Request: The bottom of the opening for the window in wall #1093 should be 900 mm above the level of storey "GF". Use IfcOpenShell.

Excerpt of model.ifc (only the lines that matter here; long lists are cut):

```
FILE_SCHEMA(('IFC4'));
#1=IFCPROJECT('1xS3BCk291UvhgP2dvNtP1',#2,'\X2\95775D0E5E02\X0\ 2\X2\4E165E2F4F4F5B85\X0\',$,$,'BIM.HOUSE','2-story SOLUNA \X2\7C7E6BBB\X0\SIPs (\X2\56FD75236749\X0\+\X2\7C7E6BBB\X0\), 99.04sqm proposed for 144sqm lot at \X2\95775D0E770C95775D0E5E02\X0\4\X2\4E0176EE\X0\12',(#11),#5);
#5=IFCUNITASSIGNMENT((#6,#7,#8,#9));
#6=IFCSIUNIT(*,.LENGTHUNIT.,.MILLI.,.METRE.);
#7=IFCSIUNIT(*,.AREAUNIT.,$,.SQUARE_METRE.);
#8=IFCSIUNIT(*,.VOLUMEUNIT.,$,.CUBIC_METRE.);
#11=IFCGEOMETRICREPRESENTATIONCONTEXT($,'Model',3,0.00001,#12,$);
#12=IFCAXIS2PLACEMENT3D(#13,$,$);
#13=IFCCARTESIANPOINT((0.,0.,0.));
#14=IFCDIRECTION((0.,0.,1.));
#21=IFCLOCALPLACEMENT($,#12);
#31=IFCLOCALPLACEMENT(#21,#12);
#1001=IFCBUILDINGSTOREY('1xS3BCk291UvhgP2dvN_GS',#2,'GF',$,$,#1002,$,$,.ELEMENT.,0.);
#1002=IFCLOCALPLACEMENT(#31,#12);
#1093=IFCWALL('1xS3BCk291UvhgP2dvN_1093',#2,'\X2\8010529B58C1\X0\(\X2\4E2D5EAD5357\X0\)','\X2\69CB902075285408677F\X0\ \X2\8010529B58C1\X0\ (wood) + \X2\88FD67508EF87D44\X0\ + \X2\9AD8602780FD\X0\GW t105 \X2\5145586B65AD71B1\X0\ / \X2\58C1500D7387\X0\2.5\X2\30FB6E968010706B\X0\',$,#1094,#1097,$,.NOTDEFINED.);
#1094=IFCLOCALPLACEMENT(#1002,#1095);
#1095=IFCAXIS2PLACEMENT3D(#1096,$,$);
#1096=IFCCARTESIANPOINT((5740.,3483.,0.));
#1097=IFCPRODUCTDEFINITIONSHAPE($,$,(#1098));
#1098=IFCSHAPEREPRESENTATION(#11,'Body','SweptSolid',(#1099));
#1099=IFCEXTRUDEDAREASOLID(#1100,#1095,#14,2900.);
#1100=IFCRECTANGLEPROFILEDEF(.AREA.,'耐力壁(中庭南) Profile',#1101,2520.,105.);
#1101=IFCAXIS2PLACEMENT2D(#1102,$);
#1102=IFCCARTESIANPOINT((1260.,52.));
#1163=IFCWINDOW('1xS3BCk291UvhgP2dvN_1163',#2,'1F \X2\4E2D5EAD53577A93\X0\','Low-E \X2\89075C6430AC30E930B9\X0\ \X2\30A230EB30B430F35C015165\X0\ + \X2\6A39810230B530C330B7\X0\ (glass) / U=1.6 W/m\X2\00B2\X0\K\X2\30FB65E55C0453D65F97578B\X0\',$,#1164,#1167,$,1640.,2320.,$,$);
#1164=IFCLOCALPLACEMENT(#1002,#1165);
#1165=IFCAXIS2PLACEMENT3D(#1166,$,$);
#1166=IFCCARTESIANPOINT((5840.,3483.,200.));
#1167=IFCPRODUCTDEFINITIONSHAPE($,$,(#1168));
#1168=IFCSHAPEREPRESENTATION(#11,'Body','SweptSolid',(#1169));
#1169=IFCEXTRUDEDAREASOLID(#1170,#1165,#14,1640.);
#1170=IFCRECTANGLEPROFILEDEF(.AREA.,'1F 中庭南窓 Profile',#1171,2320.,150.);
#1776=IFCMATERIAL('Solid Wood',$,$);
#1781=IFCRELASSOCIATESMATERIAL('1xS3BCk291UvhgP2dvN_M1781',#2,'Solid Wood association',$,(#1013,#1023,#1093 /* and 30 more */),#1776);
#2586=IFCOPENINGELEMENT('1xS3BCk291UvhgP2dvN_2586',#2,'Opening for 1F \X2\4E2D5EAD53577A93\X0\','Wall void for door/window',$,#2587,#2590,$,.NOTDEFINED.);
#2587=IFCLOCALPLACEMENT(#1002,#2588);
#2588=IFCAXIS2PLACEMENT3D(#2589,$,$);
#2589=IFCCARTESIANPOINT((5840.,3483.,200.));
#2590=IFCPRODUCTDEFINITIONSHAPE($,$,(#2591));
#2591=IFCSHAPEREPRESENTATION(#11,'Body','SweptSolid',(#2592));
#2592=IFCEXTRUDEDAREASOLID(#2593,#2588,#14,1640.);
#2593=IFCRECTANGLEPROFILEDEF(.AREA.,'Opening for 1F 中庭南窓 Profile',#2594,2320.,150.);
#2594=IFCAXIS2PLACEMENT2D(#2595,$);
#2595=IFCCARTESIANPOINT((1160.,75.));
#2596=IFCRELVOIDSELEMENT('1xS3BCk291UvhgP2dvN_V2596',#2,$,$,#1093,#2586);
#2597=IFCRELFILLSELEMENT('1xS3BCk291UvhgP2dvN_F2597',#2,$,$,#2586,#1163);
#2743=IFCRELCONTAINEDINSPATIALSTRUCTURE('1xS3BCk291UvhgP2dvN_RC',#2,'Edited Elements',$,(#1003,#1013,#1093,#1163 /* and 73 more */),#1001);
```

```python
import numpy as np
import ifcopenshell
import ifcopenshell.api.geometry
import ifcopenshell.geom
import ifcopenshell.util.element
import ifcopenshell.util.placement
import ifcopenshell.util.shape
import ifcopenshell.util.unit

model = ifcopenshell.open("model.ifc")
unit_scale = ifcopenshell.util.unit.calculate_unit_scale(model)

window = model.by_guid("1xS3BCk291UvhgP2dvN_1163")
opening = window.FillsVoids[0].RelatingOpeningElement
storey = ifcopenshell.util.element.get_container(window, ifc_class="IfcBuildingStorey")
level = ifcopenshell.util.placement.get_local_placement(storey.ObjectPlacement)[2, 3]

# The opening's origin need not be at the sill, so measure its lowest point.
shape = ifcopenshell.geom.create_shape(ifcopenshell.geom.settings(), opening)
bottom = ifcopenshell.util.shape.get_shape_bottom_elevation(shape, shape.geometry) / unit_scale
dz = level + 0.9 / unit_scale - bottom

shift = np.array([0.0, 0.0, dz])
# The window is not placed relative to its opening, so move both.
for product in (opening, window):
    matrix = ifcopenshell.util.placement.get_local_placement(product.ObjectPlacement)
    matrix[:3, 3] += shift
    ifcopenshell.api.geometry.edit_object_placement(model, product=product, matrix=matrix, is_si=False)

print(f"moved by {dz * unit_scale:+.3f} m")

model.write("model-out.ifc")
```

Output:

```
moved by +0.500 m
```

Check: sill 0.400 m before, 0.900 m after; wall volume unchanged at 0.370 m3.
